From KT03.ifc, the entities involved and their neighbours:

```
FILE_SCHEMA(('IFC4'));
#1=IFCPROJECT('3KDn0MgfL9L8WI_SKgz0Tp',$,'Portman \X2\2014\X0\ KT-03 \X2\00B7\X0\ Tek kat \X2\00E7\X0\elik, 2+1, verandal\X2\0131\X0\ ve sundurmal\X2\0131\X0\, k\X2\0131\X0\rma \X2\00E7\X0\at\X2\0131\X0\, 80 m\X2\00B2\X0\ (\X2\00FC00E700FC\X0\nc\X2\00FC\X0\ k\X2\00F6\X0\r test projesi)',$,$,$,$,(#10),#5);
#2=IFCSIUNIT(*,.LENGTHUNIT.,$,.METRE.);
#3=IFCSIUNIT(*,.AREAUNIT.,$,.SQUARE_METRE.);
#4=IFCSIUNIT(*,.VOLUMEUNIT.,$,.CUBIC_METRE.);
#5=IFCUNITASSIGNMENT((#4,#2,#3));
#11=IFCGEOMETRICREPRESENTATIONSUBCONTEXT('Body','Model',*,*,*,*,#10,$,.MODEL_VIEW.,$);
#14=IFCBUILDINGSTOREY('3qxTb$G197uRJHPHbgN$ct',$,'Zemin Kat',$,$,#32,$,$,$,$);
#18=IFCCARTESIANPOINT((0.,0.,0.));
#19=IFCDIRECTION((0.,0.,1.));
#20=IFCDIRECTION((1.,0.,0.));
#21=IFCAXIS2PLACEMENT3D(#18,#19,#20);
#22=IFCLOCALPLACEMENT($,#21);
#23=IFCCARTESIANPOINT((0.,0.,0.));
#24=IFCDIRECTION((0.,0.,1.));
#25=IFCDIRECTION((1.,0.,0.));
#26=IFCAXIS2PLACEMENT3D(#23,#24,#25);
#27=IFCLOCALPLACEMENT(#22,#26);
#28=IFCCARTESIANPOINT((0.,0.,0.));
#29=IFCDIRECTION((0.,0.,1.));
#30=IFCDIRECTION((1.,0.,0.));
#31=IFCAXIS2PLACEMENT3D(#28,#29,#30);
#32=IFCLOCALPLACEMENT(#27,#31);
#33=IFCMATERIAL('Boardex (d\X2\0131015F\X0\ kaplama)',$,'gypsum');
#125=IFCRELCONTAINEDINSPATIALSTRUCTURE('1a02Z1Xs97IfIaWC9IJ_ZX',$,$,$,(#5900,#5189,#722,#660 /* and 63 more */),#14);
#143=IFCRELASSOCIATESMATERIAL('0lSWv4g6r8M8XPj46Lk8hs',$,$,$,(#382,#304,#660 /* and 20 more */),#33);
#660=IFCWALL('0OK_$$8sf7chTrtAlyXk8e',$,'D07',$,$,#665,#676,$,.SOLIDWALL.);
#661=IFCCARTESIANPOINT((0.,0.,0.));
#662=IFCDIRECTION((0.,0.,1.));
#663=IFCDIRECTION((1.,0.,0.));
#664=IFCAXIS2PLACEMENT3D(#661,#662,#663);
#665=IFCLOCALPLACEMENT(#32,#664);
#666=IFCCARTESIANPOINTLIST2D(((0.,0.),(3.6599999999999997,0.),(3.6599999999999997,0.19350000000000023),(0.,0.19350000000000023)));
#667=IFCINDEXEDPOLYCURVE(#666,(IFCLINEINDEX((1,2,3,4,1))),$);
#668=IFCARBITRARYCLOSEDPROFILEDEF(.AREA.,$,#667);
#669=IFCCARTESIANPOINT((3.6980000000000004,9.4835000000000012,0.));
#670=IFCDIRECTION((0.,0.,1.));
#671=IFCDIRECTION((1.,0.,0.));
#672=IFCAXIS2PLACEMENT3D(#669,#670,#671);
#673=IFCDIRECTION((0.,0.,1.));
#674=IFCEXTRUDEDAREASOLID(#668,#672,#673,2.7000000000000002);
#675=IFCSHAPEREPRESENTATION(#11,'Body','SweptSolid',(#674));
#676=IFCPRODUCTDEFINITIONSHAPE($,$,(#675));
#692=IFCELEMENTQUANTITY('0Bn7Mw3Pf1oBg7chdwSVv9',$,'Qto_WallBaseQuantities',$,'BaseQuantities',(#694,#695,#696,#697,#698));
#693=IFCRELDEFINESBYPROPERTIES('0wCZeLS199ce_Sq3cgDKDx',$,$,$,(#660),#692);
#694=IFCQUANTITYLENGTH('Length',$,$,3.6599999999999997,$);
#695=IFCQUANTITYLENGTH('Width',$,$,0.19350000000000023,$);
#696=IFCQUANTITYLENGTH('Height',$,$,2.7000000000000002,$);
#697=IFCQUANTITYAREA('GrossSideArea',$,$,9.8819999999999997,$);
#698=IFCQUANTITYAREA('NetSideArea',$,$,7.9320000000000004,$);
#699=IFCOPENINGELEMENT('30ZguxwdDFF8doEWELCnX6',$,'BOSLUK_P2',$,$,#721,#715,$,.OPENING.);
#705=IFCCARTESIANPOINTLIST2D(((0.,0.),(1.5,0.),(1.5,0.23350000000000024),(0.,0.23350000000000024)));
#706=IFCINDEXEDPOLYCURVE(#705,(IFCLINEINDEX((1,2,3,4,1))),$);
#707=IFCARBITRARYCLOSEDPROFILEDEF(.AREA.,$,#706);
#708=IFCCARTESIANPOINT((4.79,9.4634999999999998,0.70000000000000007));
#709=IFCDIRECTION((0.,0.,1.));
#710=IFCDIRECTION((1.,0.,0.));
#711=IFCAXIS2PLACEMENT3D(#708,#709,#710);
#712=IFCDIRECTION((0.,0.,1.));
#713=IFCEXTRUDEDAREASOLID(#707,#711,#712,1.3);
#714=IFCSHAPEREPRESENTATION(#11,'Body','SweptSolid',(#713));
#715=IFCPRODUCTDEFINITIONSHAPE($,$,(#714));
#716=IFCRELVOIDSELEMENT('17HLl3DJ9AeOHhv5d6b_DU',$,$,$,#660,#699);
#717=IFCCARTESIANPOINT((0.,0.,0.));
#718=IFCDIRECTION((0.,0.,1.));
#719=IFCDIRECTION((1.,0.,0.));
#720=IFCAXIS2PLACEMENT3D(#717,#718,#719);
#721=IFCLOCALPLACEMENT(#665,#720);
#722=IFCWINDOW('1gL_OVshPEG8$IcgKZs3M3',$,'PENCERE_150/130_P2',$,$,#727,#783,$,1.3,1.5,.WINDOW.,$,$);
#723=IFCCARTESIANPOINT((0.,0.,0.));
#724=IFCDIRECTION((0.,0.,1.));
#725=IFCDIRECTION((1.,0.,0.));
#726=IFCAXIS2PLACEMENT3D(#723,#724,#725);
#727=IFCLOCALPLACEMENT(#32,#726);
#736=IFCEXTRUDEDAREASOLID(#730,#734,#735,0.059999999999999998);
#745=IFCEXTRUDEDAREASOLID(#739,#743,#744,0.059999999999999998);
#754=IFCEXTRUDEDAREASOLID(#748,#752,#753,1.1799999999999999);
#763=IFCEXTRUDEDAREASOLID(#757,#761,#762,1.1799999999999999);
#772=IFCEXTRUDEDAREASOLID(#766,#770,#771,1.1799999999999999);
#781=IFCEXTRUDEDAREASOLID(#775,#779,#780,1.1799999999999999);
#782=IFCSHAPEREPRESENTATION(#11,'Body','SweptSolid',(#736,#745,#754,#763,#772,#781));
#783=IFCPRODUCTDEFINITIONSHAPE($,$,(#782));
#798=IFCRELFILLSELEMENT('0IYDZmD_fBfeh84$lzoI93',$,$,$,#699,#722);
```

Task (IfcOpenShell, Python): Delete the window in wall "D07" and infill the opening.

```python
import ifcopenshell
import ifcopenshell.api.feature
import ifcopenshell.api.pset
import ifcopenshell.api.root
import ifcopenshell.geom
import ifcopenshell.util.element
import ifcopenshell.util.shape
import ifcopenshell.util.unit

model = ifcopenshell.open("KT03.ifc")
area_scale = ifcopenshell.util.unit.calculate_unit_scale(model, "AREAUNIT")
settings = ifcopenshell.geom.settings()


def volume(element):
    """Net volume in cubic metres, openings subtracted."""
    shape = ifcopenshell.geom.create_shape(settings, element)
    return ifcopenshell.util.shape.get_volume(shape.geometry)


window = model.by_guid("1gL_OVshPEG8$IcgKZs3M3")
opening = window.FillsVoids[0].RelatingOpeningElement
wall = opening.VoidsElements[0].RelatingBuildingElement
before = volume(wall)

ifcopenshell.api.root.remove_product(model, product=window)
ifcopenshell.api.feature.remove_feature(model, feature=opening)

after = volume(wall)
thickness = 0.1935  # wall thickness in metres

# Update the wall's stored quantities.
qto = model.by_id(ifcopenshell.util.element.get_pset(wall, "Qto_WallBaseQuantities", should_inherit=False)["id"])
ifcopenshell.api.pset.edit_qto(model, qto=qto, properties={"NetSideArea": after / thickness / area_scale})

print(f"wall volume {before:.3f} -> {after:.3f} m3")

model.write("KT03_rev.ifc")
```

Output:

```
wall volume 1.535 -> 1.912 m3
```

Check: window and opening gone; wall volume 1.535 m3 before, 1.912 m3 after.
